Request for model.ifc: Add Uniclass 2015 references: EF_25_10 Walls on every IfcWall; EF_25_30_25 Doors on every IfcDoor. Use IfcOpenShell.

First a look at what the model holds.

```python
import ifcopenshell

model = ifcopenshell.open("model.ifc")
print(model.schema)
print("classifications:", [c.Name for c in model.by_type("IfcClassification")])
for ifc_class in ("IfcDoor", "IfcRoof", "IfcStair", "IfcWall", "IfcWindow"):
    print(ifc_class, len(model.by_type(ifc_class)))
```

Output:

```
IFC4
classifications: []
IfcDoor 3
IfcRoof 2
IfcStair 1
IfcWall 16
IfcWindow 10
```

```python
import ifcopenshell
import ifcopenshell.api.classification

model = ifcopenshell.open("model.ifc")

system = ifcopenshell.api.classification.add_classification(model, classification="Uniclass 2015")

codes = {
    "IfcWall": ("EF_25_10", "Walls"),
    "IfcDoor": ("EF_25_30_25", "Doors"),
}
for ifc_class, (code, name) in codes.items():
    products = model.by_type(ifc_class)
    ifcopenshell.api.classification.add_reference(
        model, products=products, classification=system, identification=code, name=name
    )
    print(code, len(products))

model.write("model_updated.ifc")
```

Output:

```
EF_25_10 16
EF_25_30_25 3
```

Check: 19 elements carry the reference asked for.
